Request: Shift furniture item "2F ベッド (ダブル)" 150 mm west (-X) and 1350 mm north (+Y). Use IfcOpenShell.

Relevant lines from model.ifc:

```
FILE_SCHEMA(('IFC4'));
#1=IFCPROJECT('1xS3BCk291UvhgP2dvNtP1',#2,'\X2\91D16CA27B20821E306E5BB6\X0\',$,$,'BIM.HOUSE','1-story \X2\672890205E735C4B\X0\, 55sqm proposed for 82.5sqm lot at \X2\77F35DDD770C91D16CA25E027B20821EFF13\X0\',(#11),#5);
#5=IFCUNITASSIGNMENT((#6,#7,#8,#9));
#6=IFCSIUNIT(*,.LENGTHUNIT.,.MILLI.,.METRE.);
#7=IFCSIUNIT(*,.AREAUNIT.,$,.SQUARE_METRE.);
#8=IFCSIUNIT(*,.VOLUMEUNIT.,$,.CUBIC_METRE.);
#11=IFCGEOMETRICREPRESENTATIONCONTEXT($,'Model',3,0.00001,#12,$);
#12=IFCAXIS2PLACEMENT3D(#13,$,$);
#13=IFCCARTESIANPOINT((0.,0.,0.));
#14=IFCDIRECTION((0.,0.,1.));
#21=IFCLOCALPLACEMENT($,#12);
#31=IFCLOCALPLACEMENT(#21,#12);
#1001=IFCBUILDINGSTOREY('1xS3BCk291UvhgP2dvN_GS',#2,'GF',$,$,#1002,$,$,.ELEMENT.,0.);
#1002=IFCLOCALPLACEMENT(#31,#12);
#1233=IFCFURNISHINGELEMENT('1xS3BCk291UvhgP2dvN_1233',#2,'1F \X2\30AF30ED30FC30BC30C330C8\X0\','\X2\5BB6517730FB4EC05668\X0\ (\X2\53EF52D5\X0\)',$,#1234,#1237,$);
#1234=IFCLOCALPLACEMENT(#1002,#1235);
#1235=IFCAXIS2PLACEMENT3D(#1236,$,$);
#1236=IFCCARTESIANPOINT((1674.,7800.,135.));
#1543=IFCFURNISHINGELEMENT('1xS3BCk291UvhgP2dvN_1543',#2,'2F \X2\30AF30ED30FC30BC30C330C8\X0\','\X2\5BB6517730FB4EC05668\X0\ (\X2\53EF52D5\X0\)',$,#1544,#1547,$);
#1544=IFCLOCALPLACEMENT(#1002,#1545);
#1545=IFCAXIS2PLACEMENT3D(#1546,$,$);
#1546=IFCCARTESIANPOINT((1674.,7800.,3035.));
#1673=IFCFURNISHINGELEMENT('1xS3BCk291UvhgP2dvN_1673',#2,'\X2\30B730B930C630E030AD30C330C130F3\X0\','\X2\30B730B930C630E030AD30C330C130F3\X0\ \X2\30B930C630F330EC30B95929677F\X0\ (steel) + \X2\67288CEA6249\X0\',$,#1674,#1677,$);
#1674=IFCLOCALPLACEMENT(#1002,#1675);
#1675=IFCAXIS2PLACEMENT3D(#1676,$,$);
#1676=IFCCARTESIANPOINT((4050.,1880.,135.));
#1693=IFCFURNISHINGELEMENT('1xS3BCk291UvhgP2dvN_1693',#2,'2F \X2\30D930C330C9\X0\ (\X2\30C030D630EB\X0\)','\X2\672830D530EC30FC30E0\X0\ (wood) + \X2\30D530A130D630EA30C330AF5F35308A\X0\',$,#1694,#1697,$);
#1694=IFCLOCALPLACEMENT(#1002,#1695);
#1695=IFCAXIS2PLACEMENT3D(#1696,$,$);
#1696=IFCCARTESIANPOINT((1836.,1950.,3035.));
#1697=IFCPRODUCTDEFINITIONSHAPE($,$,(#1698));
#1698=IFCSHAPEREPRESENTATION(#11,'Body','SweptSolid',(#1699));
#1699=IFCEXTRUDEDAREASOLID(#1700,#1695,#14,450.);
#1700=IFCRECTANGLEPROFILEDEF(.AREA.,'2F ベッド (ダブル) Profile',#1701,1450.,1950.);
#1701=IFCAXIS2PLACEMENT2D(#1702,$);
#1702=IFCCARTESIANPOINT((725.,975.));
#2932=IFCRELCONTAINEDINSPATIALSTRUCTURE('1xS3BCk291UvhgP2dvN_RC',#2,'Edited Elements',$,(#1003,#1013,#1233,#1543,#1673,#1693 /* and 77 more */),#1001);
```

```python
import ifcopenshell
import ifcopenshell.api.geometry
import ifcopenshell.util.placement
import ifcopenshell.util.unit

model = ifcopenshell.open("model.ifc")
unit_scale = ifcopenshell.util.unit.calculate_unit_scale(model)

item = model.by_guid("1xS3BCk291UvhgP2dvN_1693")
matrix = ifcopenshell.util.placement.get_local_placement(item.ObjectPlacement)
matrix[0, 3] -= 0.15 / unit_scale
matrix[1, 3] += 1.35 / unit_scale
ifcopenshell.api.geometry.edit_object_placement(model, product=item, matrix=matrix, is_si=False)

print(ifcopenshell.util.placement.get_local_placement(item.ObjectPlacement).round(3) + 0.0)

model.write("model-out.ifc")
```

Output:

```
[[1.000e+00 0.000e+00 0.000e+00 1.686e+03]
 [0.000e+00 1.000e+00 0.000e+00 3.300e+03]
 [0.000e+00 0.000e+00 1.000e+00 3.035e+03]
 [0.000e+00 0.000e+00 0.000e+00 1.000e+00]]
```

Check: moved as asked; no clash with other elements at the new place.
